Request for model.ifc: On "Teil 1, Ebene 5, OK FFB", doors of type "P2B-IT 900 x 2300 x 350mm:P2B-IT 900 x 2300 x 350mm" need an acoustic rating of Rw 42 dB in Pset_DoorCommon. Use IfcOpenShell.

First a look at what the model holds.

```python
import ifcopenshell
import ifcopenshell.util.element

model = ifcopenshell.open("model.ifc")
print(model.schema)
storey = next(s for s in model.by_type("IfcBuildingStorey") if s.Name == "Teil 1, Ebene 5, OK FFB")
doors = [e for e in ifcopenshell.util.element.get_decomposition(storey) if e.is_a("IfcDoor")]
seen = {}
for e in doors:
    element_type = ifcopenshell.util.element.get_type(e)
    key = (element_type.Name if element_type != e and element_type else None, ifcopenshell.util.element.get_pset(e, "Pset_DoorCommon", "AcousticRating"))
    seen[key] = seen.get(key, 0) + 1
for (name, value), count in sorted(seen.items(), key=str):
    print(count, "x", name, "|", value)
```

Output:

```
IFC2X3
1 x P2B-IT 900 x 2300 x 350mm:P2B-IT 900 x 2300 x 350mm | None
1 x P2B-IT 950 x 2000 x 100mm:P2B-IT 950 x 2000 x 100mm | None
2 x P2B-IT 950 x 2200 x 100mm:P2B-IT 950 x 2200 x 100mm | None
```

```python
import ifcopenshell
import ifcopenshell.api.pset
import ifcopenshell.util.element

model = ifcopenshell.open("model.ifc")

storey = next(s for s in model.by_type("IfcBuildingStorey") if s.Name == "Teil 1, Ebene 5, OK FFB")
doors = [e for e in ifcopenshell.util.element.get_decomposition(storey) if e.is_a("IfcDoor")]

count = 0
for e in doors:
    element_type = ifcopenshell.util.element.get_type(e)
    if element_type in (None, e) or element_type.Name != "P2B-IT 900 x 2300 x 350mm:P2B-IT 900 x 2300 x 350mm":
        continue
    # add_pset returns the element's existing set when there is one.
    pset = ifcopenshell.api.pset.add_pset(model, product=e, name="Pset_DoorCommon")
    ifcopenshell.api.pset.edit_pset(model, pset=pset, properties={"AcousticRating": "Rw 42 dB"})
    count += 1

print(count, "doors updated")

model.write("model_updated.ifc")
```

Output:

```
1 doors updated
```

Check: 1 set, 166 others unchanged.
